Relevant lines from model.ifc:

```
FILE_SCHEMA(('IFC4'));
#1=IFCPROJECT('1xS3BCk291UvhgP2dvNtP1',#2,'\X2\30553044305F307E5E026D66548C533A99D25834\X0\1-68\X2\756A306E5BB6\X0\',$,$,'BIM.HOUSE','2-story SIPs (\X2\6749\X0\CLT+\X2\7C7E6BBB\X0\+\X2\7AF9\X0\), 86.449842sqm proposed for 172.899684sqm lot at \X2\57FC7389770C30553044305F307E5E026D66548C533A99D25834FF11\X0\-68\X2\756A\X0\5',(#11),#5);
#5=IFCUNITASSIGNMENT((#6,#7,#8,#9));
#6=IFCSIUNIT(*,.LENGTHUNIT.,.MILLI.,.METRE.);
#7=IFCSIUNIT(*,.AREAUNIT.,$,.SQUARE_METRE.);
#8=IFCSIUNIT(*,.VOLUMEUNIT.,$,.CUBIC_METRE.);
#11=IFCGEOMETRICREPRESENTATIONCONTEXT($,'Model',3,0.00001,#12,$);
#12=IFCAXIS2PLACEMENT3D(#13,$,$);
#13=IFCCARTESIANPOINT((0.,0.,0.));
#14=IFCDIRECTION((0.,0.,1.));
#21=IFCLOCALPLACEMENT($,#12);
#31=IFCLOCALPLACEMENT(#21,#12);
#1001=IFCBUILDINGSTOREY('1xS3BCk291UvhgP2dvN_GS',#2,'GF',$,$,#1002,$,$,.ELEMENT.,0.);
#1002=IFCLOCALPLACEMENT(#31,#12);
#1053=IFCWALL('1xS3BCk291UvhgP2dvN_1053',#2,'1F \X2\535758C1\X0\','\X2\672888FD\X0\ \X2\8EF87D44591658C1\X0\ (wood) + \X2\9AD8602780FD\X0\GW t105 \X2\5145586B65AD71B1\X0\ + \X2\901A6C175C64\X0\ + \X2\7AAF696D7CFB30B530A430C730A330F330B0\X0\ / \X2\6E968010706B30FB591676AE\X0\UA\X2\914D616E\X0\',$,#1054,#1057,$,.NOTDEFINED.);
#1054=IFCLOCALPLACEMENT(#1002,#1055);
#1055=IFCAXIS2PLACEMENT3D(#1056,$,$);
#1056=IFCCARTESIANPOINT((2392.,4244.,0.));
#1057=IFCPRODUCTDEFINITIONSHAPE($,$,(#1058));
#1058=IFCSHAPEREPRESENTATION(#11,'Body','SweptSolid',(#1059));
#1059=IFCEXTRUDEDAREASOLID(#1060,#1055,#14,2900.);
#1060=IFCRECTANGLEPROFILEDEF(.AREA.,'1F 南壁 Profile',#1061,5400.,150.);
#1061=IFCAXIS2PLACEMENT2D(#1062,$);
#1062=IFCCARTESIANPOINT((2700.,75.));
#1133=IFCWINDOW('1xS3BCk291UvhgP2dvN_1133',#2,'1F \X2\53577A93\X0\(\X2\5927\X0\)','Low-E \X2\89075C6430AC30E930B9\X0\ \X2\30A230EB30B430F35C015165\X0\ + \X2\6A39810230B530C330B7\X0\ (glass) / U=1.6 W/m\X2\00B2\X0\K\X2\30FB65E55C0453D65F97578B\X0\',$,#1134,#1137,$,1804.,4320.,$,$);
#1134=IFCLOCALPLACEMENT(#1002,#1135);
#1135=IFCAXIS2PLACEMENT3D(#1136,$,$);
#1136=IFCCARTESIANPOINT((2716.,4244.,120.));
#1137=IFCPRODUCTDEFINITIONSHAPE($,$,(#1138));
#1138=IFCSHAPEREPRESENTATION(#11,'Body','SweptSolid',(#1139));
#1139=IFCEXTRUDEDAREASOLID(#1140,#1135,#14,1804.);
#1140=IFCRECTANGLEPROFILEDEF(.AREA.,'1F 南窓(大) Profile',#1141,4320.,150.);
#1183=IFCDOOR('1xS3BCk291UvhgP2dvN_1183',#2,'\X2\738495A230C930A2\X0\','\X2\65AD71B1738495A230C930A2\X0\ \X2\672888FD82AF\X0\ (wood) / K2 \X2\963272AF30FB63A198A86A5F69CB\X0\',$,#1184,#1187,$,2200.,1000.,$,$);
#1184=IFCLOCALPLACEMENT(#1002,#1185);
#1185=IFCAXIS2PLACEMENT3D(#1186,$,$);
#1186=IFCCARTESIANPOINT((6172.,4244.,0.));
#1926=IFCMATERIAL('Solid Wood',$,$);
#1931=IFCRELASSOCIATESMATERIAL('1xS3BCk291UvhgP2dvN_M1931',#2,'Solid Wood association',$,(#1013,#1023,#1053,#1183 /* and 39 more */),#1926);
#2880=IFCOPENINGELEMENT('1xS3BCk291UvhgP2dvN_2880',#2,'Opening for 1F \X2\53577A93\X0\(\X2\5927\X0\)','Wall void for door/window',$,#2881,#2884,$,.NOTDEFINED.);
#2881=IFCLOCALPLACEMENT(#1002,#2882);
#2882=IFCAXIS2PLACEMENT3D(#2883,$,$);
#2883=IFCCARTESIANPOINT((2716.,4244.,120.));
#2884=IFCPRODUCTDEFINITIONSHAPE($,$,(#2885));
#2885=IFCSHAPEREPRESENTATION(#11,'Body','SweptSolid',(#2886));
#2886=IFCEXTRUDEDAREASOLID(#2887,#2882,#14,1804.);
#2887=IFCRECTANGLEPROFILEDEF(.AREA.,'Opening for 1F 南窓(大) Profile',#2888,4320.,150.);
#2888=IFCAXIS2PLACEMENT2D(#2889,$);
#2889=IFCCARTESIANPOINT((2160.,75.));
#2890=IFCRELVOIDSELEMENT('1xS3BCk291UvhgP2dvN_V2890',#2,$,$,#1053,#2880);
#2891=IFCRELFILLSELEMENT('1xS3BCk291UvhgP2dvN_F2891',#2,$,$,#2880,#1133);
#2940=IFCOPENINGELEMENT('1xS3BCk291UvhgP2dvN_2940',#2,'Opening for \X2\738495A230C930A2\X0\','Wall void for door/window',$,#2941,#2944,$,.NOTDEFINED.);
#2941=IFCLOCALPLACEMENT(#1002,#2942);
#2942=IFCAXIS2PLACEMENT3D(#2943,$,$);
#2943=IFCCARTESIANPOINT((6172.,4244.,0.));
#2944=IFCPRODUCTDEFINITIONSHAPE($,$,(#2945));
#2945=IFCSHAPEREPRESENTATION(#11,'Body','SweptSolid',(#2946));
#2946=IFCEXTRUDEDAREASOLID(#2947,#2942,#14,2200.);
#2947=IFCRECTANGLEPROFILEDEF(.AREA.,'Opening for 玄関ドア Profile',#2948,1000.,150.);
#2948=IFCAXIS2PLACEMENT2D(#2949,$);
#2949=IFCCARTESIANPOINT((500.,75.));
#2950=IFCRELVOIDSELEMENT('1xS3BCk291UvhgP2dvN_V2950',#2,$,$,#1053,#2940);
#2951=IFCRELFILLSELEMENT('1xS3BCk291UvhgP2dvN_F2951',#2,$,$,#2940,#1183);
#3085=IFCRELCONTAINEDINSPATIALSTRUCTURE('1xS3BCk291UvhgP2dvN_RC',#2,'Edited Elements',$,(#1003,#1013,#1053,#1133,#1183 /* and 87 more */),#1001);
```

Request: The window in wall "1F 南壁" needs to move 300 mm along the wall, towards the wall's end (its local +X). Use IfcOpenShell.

```python
import ifcopenshell
import ifcopenshell.api.geometry
import ifcopenshell.util.placement
import ifcopenshell.util.unit

model = ifcopenshell.open("model.ifc")
unit_scale = ifcopenshell.util.unit.calculate_unit_scale(model)

window = model.by_guid("1xS3BCk291UvhgP2dvN_1133")
opening = window.FillsVoids[0].RelatingOpeningElement
wall = opening.VoidsElements[0].RelatingBuildingElement

wall_matrix = ifcopenshell.util.placement.get_local_placement(wall.ObjectPlacement)
shift = wall_matrix[:3, 0] * 0.3 / unit_scale
before = ifcopenshell.util.placement.get_local_placement(window.ObjectPlacement)[:3, 3].copy()

# The window is not placed relative to its opening, so move both.
for product in (opening, window):
    matrix = ifcopenshell.util.placement.get_local_placement(product.ObjectPlacement)
    matrix[:3, 3] += shift
    ifcopenshell.api.geometry.edit_object_placement(model, product=product, matrix=matrix, is_si=False)

after = ifcopenshell.util.placement.get_local_placement(window.ObjectPlacement)[:3, 3]
print("window moved by", (after - before).round(3) + 0.0)

model.write("model_edited.ifc")
```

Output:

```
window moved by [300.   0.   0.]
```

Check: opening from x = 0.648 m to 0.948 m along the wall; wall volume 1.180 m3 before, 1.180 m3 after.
